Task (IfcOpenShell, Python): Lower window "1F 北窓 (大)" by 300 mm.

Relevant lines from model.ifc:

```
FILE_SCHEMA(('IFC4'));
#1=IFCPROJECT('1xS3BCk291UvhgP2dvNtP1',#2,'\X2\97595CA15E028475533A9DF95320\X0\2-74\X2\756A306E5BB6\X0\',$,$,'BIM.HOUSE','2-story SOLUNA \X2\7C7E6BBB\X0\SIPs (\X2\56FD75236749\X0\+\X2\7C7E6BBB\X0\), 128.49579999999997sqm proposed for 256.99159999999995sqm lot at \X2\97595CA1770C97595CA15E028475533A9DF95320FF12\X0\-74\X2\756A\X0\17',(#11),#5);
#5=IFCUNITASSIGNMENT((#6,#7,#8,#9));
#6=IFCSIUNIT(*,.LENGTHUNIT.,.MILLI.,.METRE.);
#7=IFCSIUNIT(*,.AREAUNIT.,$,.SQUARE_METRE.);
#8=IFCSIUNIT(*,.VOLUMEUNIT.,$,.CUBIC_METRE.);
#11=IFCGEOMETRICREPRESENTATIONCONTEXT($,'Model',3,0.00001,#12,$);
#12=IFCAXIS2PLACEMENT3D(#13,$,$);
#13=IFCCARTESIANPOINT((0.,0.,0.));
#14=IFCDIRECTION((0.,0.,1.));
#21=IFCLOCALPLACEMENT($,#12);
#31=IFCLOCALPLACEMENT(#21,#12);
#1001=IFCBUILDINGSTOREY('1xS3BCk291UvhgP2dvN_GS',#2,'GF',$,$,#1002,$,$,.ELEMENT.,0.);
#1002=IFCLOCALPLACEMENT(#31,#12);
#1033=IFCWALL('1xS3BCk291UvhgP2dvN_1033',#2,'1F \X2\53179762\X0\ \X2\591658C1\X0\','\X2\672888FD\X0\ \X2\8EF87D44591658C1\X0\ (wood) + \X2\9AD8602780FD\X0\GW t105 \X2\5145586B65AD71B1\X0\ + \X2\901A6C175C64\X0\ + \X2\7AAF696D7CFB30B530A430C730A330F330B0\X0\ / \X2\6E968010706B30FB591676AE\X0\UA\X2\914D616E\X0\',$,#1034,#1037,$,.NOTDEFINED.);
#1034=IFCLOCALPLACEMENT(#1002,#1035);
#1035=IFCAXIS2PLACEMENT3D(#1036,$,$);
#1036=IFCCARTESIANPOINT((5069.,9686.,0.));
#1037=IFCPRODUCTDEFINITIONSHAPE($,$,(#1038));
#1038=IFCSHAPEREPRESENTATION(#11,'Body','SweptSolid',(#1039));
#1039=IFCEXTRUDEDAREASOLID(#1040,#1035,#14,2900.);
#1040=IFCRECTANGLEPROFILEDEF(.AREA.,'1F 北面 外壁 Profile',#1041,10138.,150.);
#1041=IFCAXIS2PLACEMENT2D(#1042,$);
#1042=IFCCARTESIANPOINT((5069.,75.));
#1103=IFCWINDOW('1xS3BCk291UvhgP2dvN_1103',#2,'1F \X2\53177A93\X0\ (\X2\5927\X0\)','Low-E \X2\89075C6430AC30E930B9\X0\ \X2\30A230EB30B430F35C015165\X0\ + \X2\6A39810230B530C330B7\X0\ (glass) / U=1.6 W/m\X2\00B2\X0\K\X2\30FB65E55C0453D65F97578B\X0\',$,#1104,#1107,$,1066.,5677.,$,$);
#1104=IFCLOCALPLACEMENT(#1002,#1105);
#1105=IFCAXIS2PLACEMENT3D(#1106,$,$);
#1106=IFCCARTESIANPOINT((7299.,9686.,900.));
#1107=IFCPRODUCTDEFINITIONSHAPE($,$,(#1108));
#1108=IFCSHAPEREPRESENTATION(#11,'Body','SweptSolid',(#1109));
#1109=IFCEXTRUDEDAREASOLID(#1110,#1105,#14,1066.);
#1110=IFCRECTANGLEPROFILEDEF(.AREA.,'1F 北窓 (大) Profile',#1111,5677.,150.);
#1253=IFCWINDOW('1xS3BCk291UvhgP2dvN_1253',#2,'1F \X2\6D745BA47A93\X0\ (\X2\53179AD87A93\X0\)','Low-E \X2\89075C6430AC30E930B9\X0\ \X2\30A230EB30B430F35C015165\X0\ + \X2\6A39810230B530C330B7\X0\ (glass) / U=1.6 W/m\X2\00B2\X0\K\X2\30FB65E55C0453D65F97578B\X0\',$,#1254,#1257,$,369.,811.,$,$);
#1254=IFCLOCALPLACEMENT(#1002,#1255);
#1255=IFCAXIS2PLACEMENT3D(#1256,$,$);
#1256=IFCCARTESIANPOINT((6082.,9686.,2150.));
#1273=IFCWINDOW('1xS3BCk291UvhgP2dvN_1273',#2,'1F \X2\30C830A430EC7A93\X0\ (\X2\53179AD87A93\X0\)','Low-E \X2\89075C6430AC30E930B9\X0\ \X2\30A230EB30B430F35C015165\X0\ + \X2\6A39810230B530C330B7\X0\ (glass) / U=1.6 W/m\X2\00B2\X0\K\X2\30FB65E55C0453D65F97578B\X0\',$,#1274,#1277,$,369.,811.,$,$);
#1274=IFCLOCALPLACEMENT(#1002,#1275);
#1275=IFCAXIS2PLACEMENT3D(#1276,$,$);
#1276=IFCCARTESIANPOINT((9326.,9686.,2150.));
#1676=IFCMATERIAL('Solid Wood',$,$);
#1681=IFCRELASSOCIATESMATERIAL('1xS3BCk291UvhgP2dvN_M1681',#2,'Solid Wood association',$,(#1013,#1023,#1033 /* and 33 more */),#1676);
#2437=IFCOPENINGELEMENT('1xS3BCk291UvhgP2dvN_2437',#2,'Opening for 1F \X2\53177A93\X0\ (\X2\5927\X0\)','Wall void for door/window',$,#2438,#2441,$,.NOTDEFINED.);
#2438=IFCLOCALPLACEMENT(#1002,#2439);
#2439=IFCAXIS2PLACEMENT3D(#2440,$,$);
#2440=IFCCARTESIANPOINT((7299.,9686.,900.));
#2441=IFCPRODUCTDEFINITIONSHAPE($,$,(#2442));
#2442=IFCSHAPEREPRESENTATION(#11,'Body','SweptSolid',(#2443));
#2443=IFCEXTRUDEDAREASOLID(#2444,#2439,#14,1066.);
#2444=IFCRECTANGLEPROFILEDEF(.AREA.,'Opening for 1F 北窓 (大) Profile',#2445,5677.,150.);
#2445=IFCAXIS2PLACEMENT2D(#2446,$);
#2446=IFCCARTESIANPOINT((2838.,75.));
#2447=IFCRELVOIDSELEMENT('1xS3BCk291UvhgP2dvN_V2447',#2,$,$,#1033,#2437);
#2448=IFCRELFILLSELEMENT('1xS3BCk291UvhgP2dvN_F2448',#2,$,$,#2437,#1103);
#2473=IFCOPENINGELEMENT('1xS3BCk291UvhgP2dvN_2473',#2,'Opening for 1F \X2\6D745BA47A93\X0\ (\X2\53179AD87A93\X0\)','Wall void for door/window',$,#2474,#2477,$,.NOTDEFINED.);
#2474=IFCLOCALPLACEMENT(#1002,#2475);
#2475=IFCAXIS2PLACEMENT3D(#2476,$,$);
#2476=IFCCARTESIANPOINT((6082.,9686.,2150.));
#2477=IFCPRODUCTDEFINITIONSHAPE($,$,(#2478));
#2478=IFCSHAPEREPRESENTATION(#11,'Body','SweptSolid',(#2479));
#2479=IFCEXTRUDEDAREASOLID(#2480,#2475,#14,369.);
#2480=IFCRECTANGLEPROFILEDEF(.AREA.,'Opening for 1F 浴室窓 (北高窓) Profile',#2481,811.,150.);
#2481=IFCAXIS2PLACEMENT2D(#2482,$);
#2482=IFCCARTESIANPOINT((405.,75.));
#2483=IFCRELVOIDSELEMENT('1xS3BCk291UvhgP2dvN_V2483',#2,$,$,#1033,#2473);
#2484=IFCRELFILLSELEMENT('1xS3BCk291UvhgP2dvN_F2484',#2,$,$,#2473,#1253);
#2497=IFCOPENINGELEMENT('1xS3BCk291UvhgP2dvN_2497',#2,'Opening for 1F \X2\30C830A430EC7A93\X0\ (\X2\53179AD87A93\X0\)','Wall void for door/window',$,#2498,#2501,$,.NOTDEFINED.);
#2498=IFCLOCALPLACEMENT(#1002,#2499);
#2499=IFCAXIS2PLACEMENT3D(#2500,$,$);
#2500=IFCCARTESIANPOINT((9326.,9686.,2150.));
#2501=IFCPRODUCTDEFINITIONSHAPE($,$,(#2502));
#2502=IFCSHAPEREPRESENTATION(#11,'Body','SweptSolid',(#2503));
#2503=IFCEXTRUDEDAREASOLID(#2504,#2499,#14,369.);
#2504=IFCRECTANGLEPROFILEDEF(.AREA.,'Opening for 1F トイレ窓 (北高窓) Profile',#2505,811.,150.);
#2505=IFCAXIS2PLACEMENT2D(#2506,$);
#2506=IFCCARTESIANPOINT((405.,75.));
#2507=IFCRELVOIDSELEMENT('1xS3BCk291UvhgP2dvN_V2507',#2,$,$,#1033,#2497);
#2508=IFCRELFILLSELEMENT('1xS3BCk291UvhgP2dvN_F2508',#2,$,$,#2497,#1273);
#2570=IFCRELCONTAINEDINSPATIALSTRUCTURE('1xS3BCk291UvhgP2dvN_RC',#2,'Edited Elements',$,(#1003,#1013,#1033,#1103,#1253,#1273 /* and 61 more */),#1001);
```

```python
import numpy as np
import ifcopenshell
import ifcopenshell.api.geometry
import ifcopenshell.util.placement
import ifcopenshell.util.unit

model = ifcopenshell.open("model.ifc")
unit_scale = ifcopenshell.util.unit.calculate_unit_scale(model)

window = model.by_guid("1xS3BCk291UvhgP2dvN_1103")
opening = window.FillsVoids[0].RelatingOpeningElement
dz = -0.3 / unit_scale

shift = np.array([0.0, 0.0, dz])
# The window is not placed relative to its opening, so move both.
for product in (opening, window):
    matrix = ifcopenshell.util.placement.get_local_placement(product.ObjectPlacement)
    matrix[:3, 3] += shift
    ifcopenshell.api.geometry.edit_object_placement(model, product=product, matrix=matrix, is_si=False)

print(f"moved by {dz * unit_scale:+.3f} m")

model.write("model_rev.ifc")
```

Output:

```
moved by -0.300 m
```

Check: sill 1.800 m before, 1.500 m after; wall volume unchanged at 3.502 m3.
